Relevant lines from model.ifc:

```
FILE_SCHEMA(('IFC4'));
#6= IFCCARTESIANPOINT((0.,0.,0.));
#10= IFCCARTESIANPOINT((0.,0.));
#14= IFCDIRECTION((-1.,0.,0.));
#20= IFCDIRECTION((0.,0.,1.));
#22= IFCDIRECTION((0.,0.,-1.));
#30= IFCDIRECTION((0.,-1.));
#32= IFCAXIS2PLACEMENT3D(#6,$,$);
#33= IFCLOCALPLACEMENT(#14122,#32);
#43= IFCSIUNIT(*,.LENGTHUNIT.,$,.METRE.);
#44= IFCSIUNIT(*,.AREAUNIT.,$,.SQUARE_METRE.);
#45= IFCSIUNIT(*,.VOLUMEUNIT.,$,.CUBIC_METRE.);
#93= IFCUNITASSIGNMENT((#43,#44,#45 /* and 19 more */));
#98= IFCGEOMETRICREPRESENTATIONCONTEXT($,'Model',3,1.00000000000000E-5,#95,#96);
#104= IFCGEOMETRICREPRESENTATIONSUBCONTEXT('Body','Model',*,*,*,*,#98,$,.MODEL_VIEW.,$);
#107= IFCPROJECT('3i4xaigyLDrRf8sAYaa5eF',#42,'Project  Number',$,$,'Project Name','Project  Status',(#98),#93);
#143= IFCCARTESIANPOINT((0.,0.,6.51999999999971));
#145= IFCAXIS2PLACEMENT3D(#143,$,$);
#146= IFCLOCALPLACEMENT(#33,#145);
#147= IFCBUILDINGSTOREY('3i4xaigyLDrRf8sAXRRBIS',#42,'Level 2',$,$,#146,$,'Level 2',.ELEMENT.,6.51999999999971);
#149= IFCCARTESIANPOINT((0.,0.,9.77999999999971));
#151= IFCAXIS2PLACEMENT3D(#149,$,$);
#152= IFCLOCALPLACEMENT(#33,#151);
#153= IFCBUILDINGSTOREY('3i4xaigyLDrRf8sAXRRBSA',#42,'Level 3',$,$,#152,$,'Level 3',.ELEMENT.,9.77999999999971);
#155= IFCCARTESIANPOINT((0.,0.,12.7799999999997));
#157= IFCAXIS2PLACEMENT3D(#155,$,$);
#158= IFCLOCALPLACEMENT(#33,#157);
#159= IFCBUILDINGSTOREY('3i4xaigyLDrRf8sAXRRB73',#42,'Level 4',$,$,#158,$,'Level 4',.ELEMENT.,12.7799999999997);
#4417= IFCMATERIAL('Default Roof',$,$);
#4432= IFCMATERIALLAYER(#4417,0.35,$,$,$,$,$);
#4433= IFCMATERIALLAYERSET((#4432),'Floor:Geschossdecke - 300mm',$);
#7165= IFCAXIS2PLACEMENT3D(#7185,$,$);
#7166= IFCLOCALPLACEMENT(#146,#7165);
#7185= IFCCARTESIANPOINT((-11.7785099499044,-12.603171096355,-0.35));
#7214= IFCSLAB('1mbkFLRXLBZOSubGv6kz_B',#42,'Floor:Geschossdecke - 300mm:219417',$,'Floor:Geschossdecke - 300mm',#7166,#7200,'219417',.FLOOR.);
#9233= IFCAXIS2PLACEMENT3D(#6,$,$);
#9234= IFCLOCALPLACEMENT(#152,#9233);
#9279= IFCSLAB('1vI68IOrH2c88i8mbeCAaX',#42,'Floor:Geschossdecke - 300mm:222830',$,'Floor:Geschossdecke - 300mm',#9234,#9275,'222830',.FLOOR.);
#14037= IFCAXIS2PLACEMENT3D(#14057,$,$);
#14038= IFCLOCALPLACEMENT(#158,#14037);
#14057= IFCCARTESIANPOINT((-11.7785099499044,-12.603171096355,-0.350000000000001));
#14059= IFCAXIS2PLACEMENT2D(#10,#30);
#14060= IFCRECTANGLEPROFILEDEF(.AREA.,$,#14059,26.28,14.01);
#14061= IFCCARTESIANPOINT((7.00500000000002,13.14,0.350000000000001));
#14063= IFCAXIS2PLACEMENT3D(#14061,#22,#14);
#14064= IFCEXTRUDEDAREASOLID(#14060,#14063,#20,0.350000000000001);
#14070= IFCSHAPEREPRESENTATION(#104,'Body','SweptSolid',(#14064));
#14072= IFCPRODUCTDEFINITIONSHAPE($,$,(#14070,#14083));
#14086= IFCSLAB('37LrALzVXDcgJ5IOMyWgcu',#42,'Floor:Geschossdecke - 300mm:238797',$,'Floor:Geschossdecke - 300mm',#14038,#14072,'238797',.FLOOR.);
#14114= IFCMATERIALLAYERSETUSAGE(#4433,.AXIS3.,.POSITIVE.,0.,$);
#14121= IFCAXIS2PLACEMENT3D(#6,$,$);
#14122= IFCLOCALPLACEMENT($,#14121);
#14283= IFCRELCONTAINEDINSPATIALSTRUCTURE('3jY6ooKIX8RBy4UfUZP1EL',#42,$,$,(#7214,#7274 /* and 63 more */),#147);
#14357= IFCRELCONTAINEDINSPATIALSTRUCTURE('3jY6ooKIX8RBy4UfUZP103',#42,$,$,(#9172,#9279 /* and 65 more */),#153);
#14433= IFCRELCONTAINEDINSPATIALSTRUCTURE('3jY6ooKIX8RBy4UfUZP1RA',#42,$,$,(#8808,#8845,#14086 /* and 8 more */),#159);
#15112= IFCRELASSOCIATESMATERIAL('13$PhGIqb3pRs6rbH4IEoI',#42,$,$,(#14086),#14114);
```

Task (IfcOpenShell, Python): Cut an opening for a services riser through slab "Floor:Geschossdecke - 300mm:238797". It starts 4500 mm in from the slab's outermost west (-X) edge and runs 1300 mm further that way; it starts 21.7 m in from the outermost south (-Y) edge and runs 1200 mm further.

```python
import numpy as np
import ifcopenshell
import ifcopenshell.api.feature
import ifcopenshell.api.geometry
import ifcopenshell.api.root
import ifcopenshell.geom
import ifcopenshell.util.placement
import ifcopenshell.util.representation
import ifcopenshell.util.shape
import ifcopenshell.util.unit

model = ifcopenshell.open("model.ifc")
unit_scale = ifcopenshell.util.unit.calculate_unit_scale(model)
settings = ifcopenshell.geom.settings()


def volume(element):
    """Net volume in cubic metres, openings subtracted."""
    shape = ifcopenshell.geom.create_shape(settings, element)
    return ifcopenshell.util.shape.get_volume(shape.geometry)


slab = model.by_guid("37LrALzVXDcgJ5IOMyWgcu")
before = volume(slab)

# Extent in the slab's own axes, in metres. The edges named are its -X and -Y sides.
slab_shape = ifcopenshell.geom.create_shape(settings, slab)
vertices = ifcopenshell.util.shape.get_vertices(slab_shape.geometry)
x_min, y_min, bottom = vertices.min(axis=0)
top = vertices[:, 2].max()

opening = ifcopenshell.api.root.create_entity(model, ifc_class="IfcOpeningElement", name="Services riser opening", predefined_type="OPENING")
context = ifcopenshell.util.representation.get_context(model, "Model", "Body", "MODEL_VIEW")
width, depth = 1.3, 1.2
outline = [(0.0, 0.0), (width, 0.0), (width, depth), (0.0, depth), (0.0, 0.0)]
# Overshoot both faces by 50 mm so the cut is clean.
shape = ifcopenshell.api.geometry.add_slab_representation(
    model, context=context, depth=top - bottom + 0.1, polyline=outline
)
ifcopenshell.api.geometry.assign_representation(model, product=opening, representation=shape)

matrix = ifcopenshell.util.placement.get_local_placement(slab.ObjectPlacement)
matrix[:, 3] = matrix @ np.append(np.array([x_min + 4.5, y_min + 21.7, bottom - 0.05]) / unit_scale, 1.0)
ifcopenshell.api.geometry.edit_object_placement(model, product=opening, matrix=matrix, is_si=False)
ifcopenshell.api.feature.add_feature(model, feature=opening, element=slab)

after = volume(slab)

print(f"slab volume {before:.3f} -> {after:.3f} m3")

model.write("model_edited.ifc")
```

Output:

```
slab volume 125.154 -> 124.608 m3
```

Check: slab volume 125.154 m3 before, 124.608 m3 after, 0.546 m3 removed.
